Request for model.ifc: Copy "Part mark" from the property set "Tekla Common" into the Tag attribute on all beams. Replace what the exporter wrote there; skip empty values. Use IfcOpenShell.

First a look at what the model holds.

```python
import ifcopenshell
import ifcopenshell.util.element

model = ifcopenshell.open("model.ifc")
print(model.schema)
beams = model.by_type("IfcBeam")
print(len(beams), "beams")
for e in beams[:8]:
    source = ifcopenshell.util.element.get_pset(e, "Tekla Common", "Part mark")
    target = e.Tag
    print(e.id(), repr(source), repr(target), sep=" | ")
```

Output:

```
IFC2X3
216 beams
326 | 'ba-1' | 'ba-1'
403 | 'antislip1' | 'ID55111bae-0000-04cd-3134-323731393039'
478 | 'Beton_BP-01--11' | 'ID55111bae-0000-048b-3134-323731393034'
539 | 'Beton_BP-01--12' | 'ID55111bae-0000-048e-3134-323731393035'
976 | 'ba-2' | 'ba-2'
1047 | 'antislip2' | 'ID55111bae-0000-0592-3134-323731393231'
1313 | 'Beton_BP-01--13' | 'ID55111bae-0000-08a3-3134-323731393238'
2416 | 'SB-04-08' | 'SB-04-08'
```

```python
import ifcopenshell
import ifcopenshell.util.element

model = ifcopenshell.open("model.ifc")

count = 0
for e in model.by_type("IfcBeam"):
    value = ifcopenshell.util.element.get_pset(e, "Tekla Common", "Part mark")
    current = e.Tag
    if not value or not value.strip() or current == value:
        continue
    e.Tag = value
    count += 1

print(count, "beams updated")

model.write("model_rev.ifc")
```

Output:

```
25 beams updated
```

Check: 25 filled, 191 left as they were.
